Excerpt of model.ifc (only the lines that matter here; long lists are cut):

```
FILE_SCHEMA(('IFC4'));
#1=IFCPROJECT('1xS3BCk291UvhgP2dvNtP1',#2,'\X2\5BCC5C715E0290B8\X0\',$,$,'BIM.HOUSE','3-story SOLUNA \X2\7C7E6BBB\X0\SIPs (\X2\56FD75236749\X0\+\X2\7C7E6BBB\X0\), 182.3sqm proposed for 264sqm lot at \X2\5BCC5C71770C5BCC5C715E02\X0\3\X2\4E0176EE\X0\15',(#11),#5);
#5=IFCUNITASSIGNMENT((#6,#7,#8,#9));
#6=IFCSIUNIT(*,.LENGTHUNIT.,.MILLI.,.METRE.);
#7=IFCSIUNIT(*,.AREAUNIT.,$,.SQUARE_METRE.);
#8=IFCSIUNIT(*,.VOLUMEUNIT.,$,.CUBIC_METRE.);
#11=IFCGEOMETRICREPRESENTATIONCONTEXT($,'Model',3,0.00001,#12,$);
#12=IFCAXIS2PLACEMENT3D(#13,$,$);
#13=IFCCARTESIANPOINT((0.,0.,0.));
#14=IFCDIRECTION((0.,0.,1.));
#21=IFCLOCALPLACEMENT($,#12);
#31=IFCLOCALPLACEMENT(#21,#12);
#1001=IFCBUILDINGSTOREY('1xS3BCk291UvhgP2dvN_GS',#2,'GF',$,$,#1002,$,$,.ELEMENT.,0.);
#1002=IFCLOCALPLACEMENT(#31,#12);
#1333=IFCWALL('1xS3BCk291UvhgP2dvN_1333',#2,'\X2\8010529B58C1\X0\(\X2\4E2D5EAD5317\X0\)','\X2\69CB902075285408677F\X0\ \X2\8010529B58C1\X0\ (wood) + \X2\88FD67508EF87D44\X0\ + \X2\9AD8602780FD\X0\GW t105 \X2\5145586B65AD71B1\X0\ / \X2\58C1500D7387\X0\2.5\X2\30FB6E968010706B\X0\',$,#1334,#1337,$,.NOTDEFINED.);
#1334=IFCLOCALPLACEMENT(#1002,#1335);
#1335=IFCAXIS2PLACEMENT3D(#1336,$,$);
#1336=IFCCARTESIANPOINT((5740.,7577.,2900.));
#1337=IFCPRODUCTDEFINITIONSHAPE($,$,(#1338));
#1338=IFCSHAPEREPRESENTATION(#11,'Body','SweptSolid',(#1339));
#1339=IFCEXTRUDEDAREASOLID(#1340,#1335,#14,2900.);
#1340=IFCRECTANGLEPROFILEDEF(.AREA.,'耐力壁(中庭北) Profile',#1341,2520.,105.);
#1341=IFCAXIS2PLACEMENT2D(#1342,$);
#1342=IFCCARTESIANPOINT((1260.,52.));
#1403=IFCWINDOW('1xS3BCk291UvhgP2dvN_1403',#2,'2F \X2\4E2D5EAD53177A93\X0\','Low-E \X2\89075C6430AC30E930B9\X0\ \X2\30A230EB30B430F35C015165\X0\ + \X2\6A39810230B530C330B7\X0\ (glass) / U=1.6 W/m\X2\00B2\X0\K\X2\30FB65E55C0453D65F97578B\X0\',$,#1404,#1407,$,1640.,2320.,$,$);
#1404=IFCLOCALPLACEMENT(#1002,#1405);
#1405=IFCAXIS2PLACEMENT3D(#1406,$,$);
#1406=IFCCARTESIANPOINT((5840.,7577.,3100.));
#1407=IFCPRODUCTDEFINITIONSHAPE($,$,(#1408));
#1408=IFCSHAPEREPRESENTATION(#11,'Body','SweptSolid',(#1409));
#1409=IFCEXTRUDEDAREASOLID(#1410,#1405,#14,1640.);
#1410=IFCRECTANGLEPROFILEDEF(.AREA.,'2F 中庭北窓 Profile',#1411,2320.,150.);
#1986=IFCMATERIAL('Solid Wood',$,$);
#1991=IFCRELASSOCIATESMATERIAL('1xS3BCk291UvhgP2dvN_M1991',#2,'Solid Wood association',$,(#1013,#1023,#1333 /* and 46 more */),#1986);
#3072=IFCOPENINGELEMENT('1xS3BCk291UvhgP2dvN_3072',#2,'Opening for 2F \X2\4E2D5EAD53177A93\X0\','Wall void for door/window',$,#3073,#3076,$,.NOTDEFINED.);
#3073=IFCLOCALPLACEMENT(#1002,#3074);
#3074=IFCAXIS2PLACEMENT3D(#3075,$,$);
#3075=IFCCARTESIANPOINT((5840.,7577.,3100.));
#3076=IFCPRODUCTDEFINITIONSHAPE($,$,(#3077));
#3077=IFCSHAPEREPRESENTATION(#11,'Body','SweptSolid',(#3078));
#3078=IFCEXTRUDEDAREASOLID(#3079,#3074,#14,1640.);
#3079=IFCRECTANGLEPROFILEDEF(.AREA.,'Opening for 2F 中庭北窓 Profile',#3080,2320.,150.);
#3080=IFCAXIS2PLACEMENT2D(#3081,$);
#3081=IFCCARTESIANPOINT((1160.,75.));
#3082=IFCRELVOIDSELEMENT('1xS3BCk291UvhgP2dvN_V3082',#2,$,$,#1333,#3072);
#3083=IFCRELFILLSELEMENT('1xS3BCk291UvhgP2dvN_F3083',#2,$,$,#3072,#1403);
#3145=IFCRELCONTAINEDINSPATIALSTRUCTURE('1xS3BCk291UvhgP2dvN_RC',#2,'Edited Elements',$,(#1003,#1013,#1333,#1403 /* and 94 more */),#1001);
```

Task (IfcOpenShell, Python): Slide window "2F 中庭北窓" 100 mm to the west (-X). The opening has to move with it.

```python
import ifcopenshell
import ifcopenshell.api.geometry
import ifcopenshell.util.placement
import ifcopenshell.util.unit

model = ifcopenshell.open("model.ifc")
unit_scale = ifcopenshell.util.unit.calculate_unit_scale(model)

window = model.by_id(1403)
opening = window.FillsVoids[0].RelatingOpeningElement
wall = opening.VoidsElements[0].RelatingBuildingElement

wall_matrix = ifcopenshell.util.placement.get_local_placement(wall.ObjectPlacement)
shift = wall_matrix[:3, 0] * -0.1 / unit_scale
before = ifcopenshell.util.placement.get_local_placement(window.ObjectPlacement)[:3, 3].copy()

# The window is not placed relative to its opening, so move both.
for product in (opening, window):
    matrix = ifcopenshell.util.placement.get_local_placement(product.ObjectPlacement)
    matrix[:3, 3] += shift
    ifcopenshell.api.geometry.edit_object_placement(model, product=product, matrix=matrix, is_si=False)

after = ifcopenshell.util.placement.get_local_placement(window.ObjectPlacement)[:3, 3]
print("window moved by", (after - before).round(3) + 0.0)

model.write("model_updated.ifc")
```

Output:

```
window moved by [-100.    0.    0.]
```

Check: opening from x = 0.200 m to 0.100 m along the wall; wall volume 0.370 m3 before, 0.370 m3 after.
